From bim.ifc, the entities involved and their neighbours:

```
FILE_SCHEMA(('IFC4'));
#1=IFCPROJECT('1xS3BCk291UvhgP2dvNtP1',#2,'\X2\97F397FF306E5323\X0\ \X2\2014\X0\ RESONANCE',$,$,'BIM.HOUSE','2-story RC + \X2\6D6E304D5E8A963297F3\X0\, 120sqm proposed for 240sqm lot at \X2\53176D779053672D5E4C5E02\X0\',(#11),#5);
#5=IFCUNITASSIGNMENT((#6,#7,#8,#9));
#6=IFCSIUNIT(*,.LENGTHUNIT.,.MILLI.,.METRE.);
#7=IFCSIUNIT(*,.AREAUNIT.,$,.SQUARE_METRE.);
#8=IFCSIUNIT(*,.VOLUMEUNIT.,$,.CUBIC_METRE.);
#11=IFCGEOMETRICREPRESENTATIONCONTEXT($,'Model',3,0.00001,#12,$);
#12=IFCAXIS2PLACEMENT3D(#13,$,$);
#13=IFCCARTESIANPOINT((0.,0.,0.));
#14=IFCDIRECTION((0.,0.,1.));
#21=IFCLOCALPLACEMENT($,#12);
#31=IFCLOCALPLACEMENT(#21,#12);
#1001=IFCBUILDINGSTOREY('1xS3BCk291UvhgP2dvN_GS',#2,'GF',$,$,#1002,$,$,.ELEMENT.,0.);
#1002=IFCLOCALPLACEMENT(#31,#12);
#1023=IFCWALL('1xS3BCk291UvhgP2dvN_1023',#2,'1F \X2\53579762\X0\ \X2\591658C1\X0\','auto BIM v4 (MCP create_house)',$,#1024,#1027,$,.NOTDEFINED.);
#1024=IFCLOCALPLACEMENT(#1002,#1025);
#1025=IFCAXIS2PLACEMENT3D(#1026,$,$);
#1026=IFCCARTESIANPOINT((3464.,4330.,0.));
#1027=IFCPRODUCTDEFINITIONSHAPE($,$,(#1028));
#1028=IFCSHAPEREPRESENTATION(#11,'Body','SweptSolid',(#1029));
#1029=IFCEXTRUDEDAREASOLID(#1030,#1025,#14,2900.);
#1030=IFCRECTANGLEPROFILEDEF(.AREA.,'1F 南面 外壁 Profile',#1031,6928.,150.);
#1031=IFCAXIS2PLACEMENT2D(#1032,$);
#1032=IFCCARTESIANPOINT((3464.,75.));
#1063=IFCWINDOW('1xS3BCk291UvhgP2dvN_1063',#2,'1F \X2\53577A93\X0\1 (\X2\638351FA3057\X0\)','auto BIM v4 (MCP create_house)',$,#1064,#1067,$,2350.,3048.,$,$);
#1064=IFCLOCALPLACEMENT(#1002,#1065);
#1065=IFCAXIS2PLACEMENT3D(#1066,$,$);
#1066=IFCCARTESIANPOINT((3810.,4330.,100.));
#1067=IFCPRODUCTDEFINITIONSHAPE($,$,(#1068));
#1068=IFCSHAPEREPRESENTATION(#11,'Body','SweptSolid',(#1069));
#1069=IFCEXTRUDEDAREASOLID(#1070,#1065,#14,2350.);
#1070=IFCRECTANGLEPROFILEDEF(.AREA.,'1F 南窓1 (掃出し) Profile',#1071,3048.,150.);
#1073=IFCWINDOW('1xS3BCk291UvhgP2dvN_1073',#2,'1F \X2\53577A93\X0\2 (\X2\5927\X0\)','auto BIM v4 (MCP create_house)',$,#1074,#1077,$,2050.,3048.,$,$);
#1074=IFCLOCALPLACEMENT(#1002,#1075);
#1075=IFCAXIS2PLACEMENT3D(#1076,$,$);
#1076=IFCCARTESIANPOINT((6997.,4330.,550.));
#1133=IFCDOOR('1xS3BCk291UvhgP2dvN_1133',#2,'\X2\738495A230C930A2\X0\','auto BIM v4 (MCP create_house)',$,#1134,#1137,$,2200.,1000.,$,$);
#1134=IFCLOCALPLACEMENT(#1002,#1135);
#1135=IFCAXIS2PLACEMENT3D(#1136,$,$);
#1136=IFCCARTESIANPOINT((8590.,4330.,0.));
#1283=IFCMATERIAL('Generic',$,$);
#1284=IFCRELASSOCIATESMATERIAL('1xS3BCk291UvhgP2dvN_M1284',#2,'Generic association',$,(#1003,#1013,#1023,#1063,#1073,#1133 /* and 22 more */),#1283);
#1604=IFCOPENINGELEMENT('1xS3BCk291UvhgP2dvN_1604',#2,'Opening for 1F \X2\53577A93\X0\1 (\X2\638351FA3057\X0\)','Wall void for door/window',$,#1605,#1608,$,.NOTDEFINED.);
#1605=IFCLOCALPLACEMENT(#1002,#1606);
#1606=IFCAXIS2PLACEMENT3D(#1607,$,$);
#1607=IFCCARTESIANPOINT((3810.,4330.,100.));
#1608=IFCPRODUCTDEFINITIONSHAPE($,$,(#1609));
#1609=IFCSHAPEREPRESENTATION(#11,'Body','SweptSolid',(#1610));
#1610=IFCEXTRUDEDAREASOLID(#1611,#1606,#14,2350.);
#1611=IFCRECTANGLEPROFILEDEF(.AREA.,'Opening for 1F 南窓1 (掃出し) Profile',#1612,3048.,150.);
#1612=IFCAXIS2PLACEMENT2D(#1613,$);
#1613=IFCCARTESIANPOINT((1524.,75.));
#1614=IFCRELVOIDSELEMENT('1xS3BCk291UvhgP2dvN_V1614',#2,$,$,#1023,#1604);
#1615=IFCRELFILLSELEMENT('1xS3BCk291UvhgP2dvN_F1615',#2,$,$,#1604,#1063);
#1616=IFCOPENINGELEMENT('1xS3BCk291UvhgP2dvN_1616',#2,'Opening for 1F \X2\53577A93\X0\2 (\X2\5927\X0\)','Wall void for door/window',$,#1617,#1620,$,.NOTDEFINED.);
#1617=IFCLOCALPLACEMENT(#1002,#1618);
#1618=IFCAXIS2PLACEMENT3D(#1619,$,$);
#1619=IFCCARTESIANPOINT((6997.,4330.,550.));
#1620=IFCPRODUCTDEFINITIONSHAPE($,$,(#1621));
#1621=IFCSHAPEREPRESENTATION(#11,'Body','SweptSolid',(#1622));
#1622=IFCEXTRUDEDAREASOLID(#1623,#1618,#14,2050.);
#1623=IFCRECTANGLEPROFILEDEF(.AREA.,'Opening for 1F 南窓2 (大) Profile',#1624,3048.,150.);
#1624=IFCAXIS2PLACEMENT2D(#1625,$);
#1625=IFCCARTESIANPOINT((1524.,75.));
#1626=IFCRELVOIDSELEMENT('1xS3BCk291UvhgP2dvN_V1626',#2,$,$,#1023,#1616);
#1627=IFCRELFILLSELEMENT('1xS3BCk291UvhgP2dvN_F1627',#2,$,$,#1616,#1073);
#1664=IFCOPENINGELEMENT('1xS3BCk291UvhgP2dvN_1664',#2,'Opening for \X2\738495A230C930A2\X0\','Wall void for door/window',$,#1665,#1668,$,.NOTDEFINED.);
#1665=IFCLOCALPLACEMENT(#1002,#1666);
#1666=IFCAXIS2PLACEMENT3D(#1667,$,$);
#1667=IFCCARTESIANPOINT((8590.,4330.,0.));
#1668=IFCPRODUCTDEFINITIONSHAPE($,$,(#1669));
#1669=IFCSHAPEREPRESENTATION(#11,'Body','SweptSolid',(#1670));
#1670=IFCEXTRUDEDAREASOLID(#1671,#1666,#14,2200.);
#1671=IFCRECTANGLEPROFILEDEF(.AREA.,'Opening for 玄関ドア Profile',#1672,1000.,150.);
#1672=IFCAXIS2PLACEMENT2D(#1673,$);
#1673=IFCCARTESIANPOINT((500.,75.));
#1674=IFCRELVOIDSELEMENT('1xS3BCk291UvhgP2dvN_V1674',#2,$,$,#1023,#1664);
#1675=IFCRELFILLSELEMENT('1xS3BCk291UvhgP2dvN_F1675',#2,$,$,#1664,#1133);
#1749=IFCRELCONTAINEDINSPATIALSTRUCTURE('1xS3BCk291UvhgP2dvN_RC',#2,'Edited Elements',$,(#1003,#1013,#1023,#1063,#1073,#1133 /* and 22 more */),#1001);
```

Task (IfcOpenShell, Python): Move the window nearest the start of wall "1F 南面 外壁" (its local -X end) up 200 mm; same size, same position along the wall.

```python
import numpy as np
import ifcopenshell
import ifcopenshell.api.geometry
import ifcopenshell.util.placement
import ifcopenshell.util.unit

model = ifcopenshell.open("bim.ifc")
unit_scale = ifcopenshell.util.unit.calculate_unit_scale(model)

window = model.by_id(1063)
opening = window.FillsVoids[0].RelatingOpeningElement
dz = 0.2 / unit_scale

shift = np.array([0.0, 0.0, dz])
# The window is not placed relative to its opening, so move both.
for product in (opening, window):
    matrix = ifcopenshell.util.placement.get_local_placement(product.ObjectPlacement)
    matrix[:3, 3] += shift
    ifcopenshell.api.geometry.edit_object_placement(model, product=product, matrix=matrix, is_si=False)

print(f"moved by {dz * unit_scale:+.3f} m")

model.write("bim_rev.ifc")
```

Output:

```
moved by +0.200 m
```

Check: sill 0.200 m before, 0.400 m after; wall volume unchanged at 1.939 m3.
